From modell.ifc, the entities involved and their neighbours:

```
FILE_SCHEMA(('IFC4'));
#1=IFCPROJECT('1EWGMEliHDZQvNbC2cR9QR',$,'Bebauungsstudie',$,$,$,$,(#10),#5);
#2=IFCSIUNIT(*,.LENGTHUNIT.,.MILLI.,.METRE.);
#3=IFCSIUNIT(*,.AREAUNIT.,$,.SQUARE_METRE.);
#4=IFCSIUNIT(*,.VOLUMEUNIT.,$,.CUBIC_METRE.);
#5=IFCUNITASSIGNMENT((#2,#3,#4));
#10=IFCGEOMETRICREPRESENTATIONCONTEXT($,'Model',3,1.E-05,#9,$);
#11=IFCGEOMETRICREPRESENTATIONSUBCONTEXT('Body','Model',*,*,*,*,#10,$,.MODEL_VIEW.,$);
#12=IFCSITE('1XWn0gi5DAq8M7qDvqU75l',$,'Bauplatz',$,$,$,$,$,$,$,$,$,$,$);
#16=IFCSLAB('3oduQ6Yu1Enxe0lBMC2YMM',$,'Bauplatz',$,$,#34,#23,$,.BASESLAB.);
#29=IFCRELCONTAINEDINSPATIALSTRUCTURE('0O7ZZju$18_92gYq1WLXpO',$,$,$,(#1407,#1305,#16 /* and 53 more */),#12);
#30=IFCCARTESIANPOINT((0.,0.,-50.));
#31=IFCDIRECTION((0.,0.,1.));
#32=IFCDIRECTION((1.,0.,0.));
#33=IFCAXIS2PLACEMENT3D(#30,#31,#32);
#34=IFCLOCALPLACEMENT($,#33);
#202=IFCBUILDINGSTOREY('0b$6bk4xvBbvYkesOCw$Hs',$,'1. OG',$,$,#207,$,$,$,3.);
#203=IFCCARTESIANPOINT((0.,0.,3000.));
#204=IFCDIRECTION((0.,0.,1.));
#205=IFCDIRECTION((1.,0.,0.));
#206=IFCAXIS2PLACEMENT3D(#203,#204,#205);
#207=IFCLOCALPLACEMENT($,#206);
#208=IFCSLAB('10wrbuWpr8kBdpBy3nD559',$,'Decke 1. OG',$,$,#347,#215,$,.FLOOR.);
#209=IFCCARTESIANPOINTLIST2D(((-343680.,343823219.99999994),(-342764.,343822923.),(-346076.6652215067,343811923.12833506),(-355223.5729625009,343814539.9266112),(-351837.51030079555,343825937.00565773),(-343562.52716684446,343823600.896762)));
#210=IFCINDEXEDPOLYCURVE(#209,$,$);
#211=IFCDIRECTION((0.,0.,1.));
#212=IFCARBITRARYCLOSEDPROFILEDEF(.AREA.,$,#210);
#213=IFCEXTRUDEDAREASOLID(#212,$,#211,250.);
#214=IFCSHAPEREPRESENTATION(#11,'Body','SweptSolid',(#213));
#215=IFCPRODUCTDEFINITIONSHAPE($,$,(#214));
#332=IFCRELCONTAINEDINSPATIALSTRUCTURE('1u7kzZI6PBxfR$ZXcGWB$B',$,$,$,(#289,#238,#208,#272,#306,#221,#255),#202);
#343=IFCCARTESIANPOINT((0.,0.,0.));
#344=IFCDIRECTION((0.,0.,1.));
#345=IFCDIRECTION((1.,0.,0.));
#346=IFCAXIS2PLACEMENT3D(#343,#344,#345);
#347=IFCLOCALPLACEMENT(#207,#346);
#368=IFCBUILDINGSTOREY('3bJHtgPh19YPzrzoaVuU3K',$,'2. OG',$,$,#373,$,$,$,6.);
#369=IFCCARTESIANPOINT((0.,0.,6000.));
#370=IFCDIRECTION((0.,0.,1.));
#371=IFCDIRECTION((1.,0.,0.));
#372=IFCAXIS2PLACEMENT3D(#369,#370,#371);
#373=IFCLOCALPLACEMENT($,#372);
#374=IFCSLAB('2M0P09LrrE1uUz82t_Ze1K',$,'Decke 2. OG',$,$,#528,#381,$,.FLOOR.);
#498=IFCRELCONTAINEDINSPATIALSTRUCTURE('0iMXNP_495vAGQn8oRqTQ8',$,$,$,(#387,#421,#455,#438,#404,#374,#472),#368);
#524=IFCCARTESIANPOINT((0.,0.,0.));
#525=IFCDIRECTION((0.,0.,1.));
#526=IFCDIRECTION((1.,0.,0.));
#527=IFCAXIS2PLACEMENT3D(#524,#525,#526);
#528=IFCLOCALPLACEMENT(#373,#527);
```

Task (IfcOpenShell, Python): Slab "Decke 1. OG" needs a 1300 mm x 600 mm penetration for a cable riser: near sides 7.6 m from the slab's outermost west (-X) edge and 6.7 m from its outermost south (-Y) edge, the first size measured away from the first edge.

```python
import numpy as np
import ifcopenshell
import ifcopenshell.api.feature
import ifcopenshell.api.geometry
import ifcopenshell.api.root
import ifcopenshell.geom
import ifcopenshell.util.placement
import ifcopenshell.util.representation
import ifcopenshell.util.shape
import ifcopenshell.util.unit

model = ifcopenshell.open("modell.ifc")
unit_scale = ifcopenshell.util.unit.calculate_unit_scale(model)
settings = ifcopenshell.geom.settings()


def volume(element):
    """Net volume in cubic metres, openings subtracted."""
    shape = ifcopenshell.geom.create_shape(settings, element)
    return ifcopenshell.util.shape.get_volume(shape.geometry)


slab = model.by_id(208)
before = volume(slab)

# Extent in the slab's own axes, in metres. The edges named are its -X and -Y sides.
slab_shape = ifcopenshell.geom.create_shape(settings, slab)
vertices = ifcopenshell.util.shape.get_vertices(slab_shape.geometry)
x_min, y_min, bottom = vertices.min(axis=0)
top = vertices[:, 2].max()

opening = ifcopenshell.api.root.create_entity(model, ifc_class="IfcOpeningElement", name="Cable riser opening", predefined_type="OPENING")
context = ifcopenshell.util.representation.get_context(model, "Model", "Body", "MODEL_VIEW")
width, depth = 1.3, 0.6
outline = [(0.0, 0.0), (width, 0.0), (width, depth), (0.0, depth), (0.0, 0.0)]
# Overshoot both faces by 50 mm so the cut is clean.
shape = ifcopenshell.api.geometry.add_slab_representation(
    model, context=context, depth=top - bottom + 0.1, polyline=outline
)
ifcopenshell.api.geometry.assign_representation(model, product=opening, representation=shape)

matrix = ifcopenshell.util.placement.get_local_placement(slab.ObjectPlacement)
matrix[:, 3] = matrix @ np.append(np.array([x_min + 7.6, y_min + 6.7, bottom - 0.05]) / unit_scale, 1.0)
ifcopenshell.api.geometry.edit_object_placement(model, product=opening, matrix=matrix, is_si=False)
ifcopenshell.api.feature.add_feature(model, feature=opening, element=slab)

after = volume(slab)

print(f"slab volume {before:.3f} -> {after:.3f} m3")

model.write("modell_edited.ifc")
```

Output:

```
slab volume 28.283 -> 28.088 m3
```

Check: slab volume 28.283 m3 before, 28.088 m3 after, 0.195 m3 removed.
